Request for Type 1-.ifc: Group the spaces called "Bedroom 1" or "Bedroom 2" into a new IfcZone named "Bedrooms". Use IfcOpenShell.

First a look at what the model holds.

```python
import ifcopenshell

model = ifcopenshell.open("Type 1-.ifc")
print(model.schema)
seen = {}
for space in model.by_type("IfcSpace"):
    seen[space.LongName] = seen.get(space.LongName, 0) + 1
for name, count in sorted(seen.items(), key=str):
    print(count, "x", name)
print("zones:", [z.Name for z in model.by_type("IfcZone")][:20])
```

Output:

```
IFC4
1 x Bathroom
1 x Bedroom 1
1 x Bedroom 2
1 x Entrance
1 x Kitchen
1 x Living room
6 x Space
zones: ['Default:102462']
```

```python
import ifcopenshell
import ifcopenshell.api.group
import ifcopenshell.api.root

model = ifcopenshell.open("Type 1-.ifc")

names = {"Bedroom 1", "Bedroom 2"}
spaces = [s for s in model.by_type("IfcSpace") if s.LongName in names]

zone = ifcopenshell.api.root.create_entity(model, ifc_class="IfcZone", name="Bedrooms")
ifcopenshell.api.group.assign_group(model, products=spaces, group=zone)
print(len(spaces), "spaces in", zone.Name)

model.write("Type 1-_edited.ifc")
```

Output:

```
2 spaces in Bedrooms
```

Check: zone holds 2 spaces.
